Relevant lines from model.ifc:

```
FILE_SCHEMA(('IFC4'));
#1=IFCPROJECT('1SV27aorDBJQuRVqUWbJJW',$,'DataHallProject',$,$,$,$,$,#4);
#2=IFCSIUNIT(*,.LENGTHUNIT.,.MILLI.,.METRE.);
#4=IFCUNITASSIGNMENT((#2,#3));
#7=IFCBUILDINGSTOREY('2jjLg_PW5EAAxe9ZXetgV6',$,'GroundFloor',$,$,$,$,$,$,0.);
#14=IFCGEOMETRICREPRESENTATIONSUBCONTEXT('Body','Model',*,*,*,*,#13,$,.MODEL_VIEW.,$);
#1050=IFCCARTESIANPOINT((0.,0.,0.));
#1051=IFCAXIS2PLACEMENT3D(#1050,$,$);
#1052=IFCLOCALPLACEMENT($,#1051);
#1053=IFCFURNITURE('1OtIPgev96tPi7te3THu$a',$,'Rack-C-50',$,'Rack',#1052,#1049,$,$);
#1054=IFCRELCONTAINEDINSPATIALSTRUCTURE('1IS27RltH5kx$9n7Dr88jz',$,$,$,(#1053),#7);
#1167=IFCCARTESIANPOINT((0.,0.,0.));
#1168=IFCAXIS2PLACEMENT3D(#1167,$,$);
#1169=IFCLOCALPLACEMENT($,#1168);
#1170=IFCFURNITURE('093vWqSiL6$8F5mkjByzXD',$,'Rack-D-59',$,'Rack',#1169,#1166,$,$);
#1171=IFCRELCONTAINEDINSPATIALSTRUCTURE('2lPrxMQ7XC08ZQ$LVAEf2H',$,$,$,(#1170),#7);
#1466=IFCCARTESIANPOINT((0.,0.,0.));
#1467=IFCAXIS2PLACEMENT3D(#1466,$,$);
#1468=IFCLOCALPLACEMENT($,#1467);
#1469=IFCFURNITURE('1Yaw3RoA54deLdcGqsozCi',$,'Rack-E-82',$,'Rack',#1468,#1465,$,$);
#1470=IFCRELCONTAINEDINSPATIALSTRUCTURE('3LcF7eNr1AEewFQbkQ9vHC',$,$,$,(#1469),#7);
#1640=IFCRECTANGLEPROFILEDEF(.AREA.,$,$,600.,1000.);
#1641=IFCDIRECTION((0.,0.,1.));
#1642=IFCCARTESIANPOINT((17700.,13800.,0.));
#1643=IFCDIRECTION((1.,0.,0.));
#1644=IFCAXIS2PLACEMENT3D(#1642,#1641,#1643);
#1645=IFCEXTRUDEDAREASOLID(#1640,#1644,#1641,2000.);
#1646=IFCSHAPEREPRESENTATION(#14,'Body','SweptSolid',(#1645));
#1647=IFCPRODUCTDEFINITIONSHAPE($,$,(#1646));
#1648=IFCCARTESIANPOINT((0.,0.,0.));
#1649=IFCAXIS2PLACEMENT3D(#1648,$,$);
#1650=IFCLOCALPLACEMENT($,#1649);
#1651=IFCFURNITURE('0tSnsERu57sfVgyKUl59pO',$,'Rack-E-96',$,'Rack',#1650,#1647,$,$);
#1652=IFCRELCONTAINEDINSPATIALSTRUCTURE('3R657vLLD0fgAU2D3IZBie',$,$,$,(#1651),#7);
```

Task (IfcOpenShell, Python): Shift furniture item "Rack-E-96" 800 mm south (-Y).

```python
import ifcopenshell
import ifcopenshell.api.geometry
import ifcopenshell.util.placement
import ifcopenshell.util.unit

model = ifcopenshell.open("model.ifc")
unit_scale = ifcopenshell.util.unit.calculate_unit_scale(model)

item = model.by_guid("0tSnsERu57sfVgyKUl59pO")
matrix = ifcopenshell.util.placement.get_local_placement(item.ObjectPlacement)
matrix[1, 3] -= 0.8 / unit_scale
ifcopenshell.api.geometry.edit_object_placement(model, product=item, matrix=matrix, is_si=False)

print(ifcopenshell.util.placement.get_local_placement(item.ObjectPlacement).round(3) + 0.0)

model.write("model-out.ifc")
```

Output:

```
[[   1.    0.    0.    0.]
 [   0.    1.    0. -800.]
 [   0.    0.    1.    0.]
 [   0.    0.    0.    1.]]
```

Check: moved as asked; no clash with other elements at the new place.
